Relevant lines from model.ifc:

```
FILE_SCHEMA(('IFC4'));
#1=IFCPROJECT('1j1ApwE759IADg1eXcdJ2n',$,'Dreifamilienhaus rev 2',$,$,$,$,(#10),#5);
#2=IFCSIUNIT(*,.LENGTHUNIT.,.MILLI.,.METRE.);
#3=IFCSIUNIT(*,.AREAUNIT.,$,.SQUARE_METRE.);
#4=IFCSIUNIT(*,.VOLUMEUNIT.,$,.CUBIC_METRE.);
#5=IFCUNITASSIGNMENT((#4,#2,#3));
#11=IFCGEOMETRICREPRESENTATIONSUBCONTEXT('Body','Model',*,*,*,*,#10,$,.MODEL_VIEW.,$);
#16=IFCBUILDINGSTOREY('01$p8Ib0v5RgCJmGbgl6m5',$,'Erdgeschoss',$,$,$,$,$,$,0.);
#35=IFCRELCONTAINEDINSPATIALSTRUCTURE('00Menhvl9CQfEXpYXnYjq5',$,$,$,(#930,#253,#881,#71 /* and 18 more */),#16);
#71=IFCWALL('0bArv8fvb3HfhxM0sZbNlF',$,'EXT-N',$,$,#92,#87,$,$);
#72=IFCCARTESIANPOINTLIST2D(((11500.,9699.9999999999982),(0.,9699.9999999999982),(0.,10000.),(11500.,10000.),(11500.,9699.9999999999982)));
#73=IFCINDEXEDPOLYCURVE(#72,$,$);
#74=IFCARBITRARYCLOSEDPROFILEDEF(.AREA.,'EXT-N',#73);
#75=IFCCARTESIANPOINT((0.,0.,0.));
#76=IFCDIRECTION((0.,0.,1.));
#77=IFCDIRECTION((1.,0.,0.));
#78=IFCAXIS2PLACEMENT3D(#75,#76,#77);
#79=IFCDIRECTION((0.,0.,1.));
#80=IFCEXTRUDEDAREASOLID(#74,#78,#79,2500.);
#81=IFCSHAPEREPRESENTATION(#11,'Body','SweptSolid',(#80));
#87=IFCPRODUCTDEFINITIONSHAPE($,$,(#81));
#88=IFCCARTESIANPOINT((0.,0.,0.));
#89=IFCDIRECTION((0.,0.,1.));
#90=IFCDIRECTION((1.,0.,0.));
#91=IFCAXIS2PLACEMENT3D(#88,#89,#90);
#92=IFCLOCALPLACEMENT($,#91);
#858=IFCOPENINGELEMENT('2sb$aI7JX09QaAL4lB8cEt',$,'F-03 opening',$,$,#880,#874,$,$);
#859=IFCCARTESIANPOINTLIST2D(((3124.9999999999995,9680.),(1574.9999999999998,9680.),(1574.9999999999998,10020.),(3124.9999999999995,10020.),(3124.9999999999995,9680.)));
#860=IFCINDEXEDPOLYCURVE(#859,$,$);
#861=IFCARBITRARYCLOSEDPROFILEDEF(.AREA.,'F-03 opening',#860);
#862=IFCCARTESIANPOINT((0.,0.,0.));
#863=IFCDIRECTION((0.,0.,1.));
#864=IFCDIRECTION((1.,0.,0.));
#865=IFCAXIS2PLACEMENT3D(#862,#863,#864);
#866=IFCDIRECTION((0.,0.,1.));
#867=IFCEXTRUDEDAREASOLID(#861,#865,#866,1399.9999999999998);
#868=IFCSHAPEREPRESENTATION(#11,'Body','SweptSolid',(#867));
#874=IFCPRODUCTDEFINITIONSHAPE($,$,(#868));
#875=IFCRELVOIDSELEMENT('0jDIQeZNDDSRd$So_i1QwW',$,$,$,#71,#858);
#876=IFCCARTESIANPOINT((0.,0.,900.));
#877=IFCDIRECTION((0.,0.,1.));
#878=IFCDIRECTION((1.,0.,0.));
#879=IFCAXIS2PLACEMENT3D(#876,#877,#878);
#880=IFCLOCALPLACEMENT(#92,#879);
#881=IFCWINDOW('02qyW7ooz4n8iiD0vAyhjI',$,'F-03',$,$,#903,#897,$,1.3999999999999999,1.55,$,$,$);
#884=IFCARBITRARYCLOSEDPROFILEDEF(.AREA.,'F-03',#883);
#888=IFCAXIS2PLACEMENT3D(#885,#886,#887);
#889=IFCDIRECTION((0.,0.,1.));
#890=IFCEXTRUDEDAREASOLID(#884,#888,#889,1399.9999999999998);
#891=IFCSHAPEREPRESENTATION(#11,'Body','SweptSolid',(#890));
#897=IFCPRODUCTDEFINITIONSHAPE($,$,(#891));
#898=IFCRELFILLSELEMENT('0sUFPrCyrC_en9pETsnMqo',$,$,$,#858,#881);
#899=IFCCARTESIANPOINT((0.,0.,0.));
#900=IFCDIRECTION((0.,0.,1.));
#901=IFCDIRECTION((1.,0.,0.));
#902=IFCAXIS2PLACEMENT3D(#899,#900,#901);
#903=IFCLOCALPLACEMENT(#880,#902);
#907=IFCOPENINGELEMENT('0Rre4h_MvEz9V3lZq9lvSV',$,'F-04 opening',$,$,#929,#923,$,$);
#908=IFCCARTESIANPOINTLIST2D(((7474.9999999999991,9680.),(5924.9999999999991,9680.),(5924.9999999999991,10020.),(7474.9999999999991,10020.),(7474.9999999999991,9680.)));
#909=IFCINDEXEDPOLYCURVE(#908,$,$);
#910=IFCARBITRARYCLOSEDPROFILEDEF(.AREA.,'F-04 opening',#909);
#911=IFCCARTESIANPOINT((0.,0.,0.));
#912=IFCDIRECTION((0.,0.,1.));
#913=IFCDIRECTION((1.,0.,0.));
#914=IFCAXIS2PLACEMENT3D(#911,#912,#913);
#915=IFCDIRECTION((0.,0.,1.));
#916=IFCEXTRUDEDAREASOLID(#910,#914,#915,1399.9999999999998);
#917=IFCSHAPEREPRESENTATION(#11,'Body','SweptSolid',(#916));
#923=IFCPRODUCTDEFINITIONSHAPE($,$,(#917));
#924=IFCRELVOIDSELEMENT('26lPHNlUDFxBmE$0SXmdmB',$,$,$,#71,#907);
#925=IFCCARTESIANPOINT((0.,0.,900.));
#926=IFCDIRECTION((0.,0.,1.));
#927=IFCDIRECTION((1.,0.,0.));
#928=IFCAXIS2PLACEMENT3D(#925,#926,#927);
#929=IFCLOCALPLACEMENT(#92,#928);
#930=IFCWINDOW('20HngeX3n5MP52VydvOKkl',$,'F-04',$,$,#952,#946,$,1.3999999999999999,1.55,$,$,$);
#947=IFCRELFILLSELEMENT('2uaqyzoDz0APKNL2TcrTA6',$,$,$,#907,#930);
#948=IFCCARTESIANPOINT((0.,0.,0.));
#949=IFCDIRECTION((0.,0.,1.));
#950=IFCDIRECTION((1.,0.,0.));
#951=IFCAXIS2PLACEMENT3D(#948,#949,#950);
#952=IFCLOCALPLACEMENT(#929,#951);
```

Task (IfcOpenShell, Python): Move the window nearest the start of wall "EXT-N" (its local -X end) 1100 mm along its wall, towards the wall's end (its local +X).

```python
import ifcopenshell
import ifcopenshell.api.geometry
import ifcopenshell.util.placement

model = ifcopenshell.open("model.ifc")

window = model.by_guid("02qyW7ooz4n8iiD0vAyhjI")
opening = window.FillsVoids[0].RelatingOpeningElement
wall = opening.VoidsElements[0].RelatingBuildingElement

wall_matrix = ifcopenshell.util.placement.get_local_placement(wall.ObjectPlacement)
shift = wall_matrix[:3, 0] * 1100.0
before = ifcopenshell.util.placement.get_local_placement(window.ObjectPlacement)[:3, 3].copy()

# The window is placed relative to its opening, so it follows when the opening moves.
matrix = ifcopenshell.util.placement.get_local_placement(opening.ObjectPlacement)
matrix[:3, 3] += shift
ifcopenshell.api.geometry.edit_object_placement(
    model, product=opening, matrix=matrix, is_si=False, should_transform_children=True
)

after = ifcopenshell.util.placement.get_local_placement(window.ObjectPlacement)[:3, 3]
print("window moved by", (after - before).round(3) + 0.0)

model.write("model_v2.ifc")
```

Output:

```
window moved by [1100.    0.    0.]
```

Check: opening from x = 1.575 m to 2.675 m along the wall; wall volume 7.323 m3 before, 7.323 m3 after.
